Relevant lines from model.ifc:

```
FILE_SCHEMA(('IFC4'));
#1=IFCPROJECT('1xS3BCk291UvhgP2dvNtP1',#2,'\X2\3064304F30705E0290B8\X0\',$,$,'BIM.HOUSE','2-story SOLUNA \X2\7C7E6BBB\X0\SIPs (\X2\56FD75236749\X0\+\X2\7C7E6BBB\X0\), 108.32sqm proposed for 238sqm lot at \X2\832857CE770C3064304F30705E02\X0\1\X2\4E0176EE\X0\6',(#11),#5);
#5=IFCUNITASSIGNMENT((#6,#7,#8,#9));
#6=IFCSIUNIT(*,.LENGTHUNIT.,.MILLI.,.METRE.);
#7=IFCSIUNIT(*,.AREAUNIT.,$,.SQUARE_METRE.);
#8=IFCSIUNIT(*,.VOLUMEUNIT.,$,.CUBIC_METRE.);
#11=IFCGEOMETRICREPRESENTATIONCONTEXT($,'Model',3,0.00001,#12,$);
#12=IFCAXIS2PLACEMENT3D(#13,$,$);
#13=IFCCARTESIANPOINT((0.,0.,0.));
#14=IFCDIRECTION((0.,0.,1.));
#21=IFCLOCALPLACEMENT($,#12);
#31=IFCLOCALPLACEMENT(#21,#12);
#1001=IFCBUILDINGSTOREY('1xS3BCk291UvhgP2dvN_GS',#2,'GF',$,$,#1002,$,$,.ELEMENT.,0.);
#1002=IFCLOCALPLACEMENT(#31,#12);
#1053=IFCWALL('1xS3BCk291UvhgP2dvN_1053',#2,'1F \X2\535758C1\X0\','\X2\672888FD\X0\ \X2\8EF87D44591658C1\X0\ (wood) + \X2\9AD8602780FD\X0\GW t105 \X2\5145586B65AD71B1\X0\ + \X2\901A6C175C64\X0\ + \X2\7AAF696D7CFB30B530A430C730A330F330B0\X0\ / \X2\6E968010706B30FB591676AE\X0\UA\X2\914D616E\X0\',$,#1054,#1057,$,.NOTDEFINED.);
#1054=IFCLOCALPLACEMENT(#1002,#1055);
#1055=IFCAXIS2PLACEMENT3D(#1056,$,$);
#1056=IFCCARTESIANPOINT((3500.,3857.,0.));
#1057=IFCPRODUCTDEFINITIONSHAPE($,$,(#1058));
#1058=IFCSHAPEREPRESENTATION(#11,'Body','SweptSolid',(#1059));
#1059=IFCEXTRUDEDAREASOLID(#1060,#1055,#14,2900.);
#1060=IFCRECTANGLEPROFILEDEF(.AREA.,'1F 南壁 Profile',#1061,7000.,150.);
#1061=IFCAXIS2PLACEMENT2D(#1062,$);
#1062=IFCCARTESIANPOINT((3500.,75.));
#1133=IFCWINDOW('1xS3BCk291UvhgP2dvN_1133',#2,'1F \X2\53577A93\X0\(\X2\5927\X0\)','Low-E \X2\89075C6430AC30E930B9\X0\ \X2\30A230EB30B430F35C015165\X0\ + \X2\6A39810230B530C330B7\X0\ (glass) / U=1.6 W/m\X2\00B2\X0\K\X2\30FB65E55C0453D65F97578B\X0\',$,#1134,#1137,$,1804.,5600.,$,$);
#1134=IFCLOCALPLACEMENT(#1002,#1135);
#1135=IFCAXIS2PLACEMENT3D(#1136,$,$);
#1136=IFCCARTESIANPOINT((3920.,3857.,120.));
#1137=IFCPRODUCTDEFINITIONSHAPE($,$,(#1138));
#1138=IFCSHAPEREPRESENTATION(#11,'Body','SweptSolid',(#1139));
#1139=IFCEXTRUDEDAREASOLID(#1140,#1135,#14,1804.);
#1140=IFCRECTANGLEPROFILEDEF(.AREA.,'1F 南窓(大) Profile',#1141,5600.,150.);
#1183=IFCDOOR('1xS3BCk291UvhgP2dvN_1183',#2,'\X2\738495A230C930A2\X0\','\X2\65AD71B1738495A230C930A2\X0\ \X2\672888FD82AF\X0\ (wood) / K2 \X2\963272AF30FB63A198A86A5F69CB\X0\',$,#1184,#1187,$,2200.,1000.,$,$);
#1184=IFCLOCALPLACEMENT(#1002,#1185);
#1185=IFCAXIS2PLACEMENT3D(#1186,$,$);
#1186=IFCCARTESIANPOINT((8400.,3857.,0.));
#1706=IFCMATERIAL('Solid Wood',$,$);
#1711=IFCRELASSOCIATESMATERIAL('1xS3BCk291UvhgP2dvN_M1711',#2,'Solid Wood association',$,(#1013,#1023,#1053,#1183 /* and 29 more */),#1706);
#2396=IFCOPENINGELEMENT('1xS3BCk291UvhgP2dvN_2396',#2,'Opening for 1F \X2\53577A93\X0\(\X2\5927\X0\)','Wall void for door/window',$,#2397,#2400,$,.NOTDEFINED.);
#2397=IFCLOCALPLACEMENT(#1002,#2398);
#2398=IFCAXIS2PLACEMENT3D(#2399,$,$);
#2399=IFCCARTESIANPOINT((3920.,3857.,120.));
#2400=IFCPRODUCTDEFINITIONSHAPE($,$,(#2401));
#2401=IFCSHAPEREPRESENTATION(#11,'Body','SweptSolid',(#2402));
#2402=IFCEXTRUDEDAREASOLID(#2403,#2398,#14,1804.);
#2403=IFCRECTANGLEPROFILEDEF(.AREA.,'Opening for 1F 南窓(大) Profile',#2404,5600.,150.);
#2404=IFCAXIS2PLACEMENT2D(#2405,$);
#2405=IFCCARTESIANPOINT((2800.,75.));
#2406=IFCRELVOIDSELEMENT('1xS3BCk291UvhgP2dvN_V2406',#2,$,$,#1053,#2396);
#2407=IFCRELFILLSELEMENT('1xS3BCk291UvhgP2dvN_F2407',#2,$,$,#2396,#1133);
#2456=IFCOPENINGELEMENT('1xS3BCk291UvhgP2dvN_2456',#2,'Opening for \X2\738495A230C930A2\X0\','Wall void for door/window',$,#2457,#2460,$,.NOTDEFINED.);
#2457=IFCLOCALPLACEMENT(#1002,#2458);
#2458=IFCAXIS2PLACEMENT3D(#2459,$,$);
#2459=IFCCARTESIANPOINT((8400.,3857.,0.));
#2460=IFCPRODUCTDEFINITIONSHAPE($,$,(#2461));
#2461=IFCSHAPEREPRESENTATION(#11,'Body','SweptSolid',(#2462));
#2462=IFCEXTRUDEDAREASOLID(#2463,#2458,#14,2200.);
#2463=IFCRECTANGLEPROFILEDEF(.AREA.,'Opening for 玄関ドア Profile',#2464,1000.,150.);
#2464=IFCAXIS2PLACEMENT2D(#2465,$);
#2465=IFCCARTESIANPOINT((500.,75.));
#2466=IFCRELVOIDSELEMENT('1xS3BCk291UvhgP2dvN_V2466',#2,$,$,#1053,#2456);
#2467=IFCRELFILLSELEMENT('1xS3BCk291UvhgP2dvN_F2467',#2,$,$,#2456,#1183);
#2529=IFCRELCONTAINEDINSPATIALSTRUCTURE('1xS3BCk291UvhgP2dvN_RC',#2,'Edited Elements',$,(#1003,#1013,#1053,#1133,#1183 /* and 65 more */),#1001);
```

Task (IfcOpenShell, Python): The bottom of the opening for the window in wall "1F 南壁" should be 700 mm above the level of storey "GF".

```python
import numpy as np
import ifcopenshell
import ifcopenshell.api.geometry
import ifcopenshell.geom
import ifcopenshell.util.element
import ifcopenshell.util.placement
import ifcopenshell.util.shape
import ifcopenshell.util.unit

model = ifcopenshell.open("model.ifc")
unit_scale = ifcopenshell.util.unit.calculate_unit_scale(model)

window = model.by_guid("1xS3BCk291UvhgP2dvN_1133")
opening = window.FillsVoids[0].RelatingOpeningElement
storey = ifcopenshell.util.element.get_container(window, ifc_class="IfcBuildingStorey")
level = ifcopenshell.util.placement.get_local_placement(storey.ObjectPlacement)[2, 3]

# The opening's origin need not be at the sill, so measure its lowest point.
shape = ifcopenshell.geom.create_shape(ifcopenshell.geom.settings(), opening)
bottom = ifcopenshell.util.shape.get_shape_bottom_elevation(shape, shape.geometry) / unit_scale
dz = level + 0.7 / unit_scale - bottom

shift = np.array([0.0, 0.0, dz])
# The window is not placed relative to its opening, so move both.
for product in (opening, window):
    matrix = ifcopenshell.util.placement.get_local_placement(product.ObjectPlacement)
    matrix[:3, 3] += shift
    ifcopenshell.api.geometry.edit_object_placement(model, product=product, matrix=matrix, is_si=False)

print(f"moved by {dz * unit_scale:+.3f} m")

model.write("model_edited.ifc")
```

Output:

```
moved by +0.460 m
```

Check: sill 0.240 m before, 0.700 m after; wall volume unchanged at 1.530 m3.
